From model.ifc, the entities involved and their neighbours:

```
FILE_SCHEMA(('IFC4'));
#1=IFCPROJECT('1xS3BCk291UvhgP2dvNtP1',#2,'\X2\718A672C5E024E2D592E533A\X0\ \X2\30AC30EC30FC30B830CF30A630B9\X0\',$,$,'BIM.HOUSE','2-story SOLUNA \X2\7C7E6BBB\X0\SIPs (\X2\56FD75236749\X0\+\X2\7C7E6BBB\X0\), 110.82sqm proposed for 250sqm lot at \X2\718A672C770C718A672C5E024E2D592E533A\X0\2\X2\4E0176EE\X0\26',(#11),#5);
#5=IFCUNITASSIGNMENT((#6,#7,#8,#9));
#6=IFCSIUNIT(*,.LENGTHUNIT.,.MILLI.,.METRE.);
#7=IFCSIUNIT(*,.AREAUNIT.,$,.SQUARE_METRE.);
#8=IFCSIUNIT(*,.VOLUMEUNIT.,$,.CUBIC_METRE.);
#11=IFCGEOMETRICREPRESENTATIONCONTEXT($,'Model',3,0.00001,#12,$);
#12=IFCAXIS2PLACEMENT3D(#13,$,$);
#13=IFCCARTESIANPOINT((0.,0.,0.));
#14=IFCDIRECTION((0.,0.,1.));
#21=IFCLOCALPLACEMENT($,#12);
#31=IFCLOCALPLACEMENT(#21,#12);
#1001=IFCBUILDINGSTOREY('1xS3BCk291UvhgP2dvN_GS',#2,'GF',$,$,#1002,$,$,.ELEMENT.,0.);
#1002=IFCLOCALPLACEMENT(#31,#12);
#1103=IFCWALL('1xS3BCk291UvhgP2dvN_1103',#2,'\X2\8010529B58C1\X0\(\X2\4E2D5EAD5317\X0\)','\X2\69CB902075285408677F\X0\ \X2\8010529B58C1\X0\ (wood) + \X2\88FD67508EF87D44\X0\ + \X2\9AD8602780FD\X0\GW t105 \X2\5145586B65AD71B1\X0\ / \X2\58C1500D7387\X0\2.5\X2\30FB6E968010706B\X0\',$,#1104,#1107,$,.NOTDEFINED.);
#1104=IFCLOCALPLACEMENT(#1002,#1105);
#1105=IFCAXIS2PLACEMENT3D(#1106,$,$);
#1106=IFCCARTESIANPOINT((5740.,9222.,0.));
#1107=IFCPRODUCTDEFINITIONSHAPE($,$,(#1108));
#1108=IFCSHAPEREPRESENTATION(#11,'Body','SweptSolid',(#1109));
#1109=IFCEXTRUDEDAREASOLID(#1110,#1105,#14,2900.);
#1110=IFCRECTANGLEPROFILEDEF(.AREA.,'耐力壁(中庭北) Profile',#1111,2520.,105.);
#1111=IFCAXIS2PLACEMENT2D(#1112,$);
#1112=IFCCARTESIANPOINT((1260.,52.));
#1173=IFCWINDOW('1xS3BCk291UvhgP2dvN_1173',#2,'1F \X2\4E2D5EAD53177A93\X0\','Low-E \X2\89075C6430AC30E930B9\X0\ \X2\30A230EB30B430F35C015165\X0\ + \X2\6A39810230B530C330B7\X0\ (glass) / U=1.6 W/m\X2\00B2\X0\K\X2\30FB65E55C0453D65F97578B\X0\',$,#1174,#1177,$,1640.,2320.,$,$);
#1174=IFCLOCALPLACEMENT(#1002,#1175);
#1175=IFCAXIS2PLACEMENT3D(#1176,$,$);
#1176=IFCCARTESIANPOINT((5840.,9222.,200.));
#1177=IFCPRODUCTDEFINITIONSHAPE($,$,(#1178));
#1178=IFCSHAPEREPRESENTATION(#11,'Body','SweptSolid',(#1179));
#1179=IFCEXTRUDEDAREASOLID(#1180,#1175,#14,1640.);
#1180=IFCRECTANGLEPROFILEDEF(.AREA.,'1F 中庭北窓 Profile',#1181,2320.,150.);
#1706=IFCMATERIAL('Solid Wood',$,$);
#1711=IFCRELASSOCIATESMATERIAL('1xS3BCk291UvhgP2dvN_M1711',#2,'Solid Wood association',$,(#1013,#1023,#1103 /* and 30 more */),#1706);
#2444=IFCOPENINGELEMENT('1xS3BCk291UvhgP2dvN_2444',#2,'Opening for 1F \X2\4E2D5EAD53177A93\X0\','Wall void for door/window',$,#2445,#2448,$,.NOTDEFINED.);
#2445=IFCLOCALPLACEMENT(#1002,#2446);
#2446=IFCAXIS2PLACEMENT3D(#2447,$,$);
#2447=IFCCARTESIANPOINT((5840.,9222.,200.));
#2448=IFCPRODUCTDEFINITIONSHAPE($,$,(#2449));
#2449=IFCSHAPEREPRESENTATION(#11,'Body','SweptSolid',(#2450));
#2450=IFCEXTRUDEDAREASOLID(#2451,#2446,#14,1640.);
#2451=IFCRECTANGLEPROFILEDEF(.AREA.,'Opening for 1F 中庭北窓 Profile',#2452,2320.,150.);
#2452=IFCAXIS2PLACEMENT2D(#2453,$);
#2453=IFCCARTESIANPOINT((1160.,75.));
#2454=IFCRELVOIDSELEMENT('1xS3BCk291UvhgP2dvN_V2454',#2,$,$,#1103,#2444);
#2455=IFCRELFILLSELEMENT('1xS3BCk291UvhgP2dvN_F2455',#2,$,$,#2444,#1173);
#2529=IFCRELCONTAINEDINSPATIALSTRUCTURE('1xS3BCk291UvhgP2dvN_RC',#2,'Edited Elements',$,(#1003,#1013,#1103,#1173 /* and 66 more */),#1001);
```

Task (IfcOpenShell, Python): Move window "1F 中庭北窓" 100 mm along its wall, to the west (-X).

```python
import ifcopenshell
import ifcopenshell.api.geometry
import ifcopenshell.util.placement

model = ifcopenshell.open("model.ifc")

window = model.by_guid("1xS3BCk291UvhgP2dvN_1173")
opening = window.FillsVoids[0].RelatingOpeningElement
wall = opening.VoidsElements[0].RelatingBuildingElement

wall_matrix = ifcopenshell.util.placement.get_local_placement(wall.ObjectPlacement)
shift = wall_matrix[:3, 0] * -100.0
before = ifcopenshell.util.placement.get_local_placement(window.ObjectPlacement)[:3, 3].copy()

# The window is not placed relative to its opening, so move both.
for product in (opening, window):
    matrix = ifcopenshell.util.placement.get_local_placement(product.ObjectPlacement)
    matrix[:3, 3] += shift
    ifcopenshell.api.geometry.edit_object_placement(model, product=product, matrix=matrix, is_si=False)

after = ifcopenshell.util.placement.get_local_placement(window.ObjectPlacement)[:3, 3]
print("window moved by", (after - before).round(3) + 0.0)

model.write("model_v2.ifc")
```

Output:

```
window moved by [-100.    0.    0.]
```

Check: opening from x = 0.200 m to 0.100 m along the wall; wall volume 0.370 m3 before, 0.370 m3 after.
